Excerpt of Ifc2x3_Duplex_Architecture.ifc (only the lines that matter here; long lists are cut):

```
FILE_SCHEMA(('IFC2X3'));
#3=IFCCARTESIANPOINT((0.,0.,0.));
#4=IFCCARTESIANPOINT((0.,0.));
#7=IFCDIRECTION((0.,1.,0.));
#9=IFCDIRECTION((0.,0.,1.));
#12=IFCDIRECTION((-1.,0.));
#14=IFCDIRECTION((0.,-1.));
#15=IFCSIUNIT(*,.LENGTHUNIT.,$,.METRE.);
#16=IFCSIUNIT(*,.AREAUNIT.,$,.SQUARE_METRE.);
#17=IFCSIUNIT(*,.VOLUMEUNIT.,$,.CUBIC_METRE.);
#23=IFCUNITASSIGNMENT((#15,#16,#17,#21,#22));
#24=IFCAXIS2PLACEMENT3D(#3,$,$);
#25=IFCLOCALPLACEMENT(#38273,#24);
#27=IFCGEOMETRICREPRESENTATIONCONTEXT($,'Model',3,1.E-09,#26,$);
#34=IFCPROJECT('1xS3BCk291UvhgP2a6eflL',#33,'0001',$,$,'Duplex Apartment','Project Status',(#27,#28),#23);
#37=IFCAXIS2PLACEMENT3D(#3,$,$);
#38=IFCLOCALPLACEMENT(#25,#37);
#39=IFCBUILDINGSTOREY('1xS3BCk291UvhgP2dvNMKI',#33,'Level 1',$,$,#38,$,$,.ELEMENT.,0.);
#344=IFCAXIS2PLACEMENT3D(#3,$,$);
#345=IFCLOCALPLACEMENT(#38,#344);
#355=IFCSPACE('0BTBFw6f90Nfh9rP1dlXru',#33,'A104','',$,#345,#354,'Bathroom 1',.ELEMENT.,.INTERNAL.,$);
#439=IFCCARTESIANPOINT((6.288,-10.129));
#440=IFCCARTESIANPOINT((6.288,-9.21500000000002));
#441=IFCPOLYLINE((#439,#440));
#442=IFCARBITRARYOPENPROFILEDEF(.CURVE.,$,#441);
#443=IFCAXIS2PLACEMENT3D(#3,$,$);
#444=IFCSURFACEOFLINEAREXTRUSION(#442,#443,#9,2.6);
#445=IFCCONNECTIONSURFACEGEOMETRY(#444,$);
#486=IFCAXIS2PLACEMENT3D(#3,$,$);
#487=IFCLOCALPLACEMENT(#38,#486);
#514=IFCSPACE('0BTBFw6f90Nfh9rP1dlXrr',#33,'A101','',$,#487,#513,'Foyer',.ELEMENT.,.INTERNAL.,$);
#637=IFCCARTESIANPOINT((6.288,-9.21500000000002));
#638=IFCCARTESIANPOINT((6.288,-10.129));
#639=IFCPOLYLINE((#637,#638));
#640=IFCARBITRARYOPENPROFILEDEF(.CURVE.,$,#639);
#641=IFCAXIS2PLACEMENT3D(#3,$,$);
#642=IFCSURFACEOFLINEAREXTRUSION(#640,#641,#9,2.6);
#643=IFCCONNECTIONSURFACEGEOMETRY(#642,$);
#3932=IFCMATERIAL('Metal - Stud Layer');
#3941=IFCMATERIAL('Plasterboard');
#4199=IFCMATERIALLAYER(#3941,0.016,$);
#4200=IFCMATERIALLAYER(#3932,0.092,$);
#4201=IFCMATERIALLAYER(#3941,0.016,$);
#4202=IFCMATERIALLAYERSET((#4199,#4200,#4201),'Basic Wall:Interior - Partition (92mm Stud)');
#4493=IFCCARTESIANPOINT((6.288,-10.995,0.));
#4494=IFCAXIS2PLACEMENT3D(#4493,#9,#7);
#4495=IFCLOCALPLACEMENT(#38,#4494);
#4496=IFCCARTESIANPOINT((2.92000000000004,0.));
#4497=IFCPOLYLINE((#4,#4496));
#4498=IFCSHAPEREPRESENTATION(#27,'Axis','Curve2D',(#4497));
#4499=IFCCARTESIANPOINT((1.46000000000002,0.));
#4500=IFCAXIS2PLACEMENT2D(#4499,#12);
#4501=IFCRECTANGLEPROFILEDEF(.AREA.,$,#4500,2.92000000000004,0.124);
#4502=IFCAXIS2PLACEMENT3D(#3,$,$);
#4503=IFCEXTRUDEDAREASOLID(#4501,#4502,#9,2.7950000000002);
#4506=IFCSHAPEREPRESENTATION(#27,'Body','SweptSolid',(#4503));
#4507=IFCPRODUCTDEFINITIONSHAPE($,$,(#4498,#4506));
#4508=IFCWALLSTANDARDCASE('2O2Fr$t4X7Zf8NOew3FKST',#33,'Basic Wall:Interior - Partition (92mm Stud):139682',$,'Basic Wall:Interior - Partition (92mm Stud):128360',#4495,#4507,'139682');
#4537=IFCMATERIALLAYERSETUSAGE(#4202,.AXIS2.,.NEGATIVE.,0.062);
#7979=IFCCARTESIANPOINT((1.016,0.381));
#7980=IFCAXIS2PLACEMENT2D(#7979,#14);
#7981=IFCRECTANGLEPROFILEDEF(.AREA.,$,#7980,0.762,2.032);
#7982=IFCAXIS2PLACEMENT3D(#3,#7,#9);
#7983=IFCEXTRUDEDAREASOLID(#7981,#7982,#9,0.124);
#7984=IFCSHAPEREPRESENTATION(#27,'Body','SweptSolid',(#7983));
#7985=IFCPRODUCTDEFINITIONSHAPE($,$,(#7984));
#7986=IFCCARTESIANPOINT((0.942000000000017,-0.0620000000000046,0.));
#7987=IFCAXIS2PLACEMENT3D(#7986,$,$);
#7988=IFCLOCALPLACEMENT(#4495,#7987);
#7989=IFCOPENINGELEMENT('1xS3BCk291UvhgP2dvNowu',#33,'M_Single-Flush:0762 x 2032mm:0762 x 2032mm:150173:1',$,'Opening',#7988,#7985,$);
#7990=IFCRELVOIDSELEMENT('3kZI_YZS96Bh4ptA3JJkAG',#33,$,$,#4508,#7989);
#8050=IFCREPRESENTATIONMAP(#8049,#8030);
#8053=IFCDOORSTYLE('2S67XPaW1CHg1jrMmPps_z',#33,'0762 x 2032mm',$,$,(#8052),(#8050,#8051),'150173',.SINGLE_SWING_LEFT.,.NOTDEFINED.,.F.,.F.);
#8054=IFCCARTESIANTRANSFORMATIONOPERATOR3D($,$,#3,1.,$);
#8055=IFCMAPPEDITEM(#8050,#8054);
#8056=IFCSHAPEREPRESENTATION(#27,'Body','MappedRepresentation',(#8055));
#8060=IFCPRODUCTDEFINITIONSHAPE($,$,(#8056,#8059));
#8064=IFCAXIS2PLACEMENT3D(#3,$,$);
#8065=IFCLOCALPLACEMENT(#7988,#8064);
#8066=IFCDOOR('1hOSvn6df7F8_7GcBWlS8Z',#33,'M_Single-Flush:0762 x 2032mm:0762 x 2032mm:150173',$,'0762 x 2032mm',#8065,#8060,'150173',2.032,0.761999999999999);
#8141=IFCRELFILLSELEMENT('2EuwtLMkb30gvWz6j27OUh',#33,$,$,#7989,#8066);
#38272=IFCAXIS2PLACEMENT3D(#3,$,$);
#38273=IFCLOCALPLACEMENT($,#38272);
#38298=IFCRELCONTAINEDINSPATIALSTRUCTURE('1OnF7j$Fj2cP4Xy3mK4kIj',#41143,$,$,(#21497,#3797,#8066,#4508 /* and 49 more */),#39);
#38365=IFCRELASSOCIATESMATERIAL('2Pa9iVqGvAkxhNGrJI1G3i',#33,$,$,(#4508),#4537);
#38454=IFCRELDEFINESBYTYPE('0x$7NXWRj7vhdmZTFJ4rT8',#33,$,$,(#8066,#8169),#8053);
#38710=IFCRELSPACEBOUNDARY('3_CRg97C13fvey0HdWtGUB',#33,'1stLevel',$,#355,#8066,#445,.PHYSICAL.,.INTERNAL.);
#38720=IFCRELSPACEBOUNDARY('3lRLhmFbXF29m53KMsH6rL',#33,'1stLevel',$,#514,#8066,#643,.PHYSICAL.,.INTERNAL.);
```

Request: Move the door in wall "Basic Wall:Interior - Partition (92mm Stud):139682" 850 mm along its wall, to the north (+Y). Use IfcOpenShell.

```python
import numpy as np
import ifcopenshell
import ifcopenshell.api.geometry
import ifcopenshell.util.placement

model = ifcopenshell.open("Ifc2x3_Duplex_Architecture.ifc")

door = model.by_guid("1hOSvn6df7F8_7GcBWlS8Z")
opening = door.FillsVoids[0].RelatingOpeningElement
wall = opening.VoidsElements[0].RelatingBuildingElement

wall_matrix = ifcopenshell.util.placement.get_local_placement(wall.ObjectPlacement)
shift = wall_matrix[:3, 0] * 0.85
before = ifcopenshell.util.placement.get_local_placement(door.ObjectPlacement)[:3, 3].copy()

# The door is placed relative to its opening, so it follows when the opening moves.
matrix = ifcopenshell.util.placement.get_local_placement(opening.ObjectPlacement)
matrix[:3, 3] += shift
ifcopenshell.api.geometry.edit_object_placement(
    model, product=opening, matrix=matrix, is_si=False, should_transform_children=True
)

# Space boundary surfaces are stored in each space's coordinates; move them too.
for rel in door.ProvidesBoundaries:
    if not rel.ConnectionGeometry:
        continue
    surface = rel.ConnectionGeometry.SurfaceOnRelatingElement
    space_matrix = ifcopenshell.util.placement.get_local_placement(rel.RelatingSpace.ObjectPlacement)
    point = np.array(surface.Position.Location.Coordinates) + space_matrix[:3, :3].T @ shift
    surface.Position = model.createIfcAxis2Placement3D(
        model.createIfcCartesianPoint(point.tolist()), surface.Position.Axis, surface.Position.RefDirection
    )

after = ifcopenshell.util.placement.get_local_placement(door.ObjectPlacement)[:3, 3]
print("door moved by", (after - before).round(3) + 0.0)

model.write("Ifc2x3_Duplex_Architecture_rev.ifc")
```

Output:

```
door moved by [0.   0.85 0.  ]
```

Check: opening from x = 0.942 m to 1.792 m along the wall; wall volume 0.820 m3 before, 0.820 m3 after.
